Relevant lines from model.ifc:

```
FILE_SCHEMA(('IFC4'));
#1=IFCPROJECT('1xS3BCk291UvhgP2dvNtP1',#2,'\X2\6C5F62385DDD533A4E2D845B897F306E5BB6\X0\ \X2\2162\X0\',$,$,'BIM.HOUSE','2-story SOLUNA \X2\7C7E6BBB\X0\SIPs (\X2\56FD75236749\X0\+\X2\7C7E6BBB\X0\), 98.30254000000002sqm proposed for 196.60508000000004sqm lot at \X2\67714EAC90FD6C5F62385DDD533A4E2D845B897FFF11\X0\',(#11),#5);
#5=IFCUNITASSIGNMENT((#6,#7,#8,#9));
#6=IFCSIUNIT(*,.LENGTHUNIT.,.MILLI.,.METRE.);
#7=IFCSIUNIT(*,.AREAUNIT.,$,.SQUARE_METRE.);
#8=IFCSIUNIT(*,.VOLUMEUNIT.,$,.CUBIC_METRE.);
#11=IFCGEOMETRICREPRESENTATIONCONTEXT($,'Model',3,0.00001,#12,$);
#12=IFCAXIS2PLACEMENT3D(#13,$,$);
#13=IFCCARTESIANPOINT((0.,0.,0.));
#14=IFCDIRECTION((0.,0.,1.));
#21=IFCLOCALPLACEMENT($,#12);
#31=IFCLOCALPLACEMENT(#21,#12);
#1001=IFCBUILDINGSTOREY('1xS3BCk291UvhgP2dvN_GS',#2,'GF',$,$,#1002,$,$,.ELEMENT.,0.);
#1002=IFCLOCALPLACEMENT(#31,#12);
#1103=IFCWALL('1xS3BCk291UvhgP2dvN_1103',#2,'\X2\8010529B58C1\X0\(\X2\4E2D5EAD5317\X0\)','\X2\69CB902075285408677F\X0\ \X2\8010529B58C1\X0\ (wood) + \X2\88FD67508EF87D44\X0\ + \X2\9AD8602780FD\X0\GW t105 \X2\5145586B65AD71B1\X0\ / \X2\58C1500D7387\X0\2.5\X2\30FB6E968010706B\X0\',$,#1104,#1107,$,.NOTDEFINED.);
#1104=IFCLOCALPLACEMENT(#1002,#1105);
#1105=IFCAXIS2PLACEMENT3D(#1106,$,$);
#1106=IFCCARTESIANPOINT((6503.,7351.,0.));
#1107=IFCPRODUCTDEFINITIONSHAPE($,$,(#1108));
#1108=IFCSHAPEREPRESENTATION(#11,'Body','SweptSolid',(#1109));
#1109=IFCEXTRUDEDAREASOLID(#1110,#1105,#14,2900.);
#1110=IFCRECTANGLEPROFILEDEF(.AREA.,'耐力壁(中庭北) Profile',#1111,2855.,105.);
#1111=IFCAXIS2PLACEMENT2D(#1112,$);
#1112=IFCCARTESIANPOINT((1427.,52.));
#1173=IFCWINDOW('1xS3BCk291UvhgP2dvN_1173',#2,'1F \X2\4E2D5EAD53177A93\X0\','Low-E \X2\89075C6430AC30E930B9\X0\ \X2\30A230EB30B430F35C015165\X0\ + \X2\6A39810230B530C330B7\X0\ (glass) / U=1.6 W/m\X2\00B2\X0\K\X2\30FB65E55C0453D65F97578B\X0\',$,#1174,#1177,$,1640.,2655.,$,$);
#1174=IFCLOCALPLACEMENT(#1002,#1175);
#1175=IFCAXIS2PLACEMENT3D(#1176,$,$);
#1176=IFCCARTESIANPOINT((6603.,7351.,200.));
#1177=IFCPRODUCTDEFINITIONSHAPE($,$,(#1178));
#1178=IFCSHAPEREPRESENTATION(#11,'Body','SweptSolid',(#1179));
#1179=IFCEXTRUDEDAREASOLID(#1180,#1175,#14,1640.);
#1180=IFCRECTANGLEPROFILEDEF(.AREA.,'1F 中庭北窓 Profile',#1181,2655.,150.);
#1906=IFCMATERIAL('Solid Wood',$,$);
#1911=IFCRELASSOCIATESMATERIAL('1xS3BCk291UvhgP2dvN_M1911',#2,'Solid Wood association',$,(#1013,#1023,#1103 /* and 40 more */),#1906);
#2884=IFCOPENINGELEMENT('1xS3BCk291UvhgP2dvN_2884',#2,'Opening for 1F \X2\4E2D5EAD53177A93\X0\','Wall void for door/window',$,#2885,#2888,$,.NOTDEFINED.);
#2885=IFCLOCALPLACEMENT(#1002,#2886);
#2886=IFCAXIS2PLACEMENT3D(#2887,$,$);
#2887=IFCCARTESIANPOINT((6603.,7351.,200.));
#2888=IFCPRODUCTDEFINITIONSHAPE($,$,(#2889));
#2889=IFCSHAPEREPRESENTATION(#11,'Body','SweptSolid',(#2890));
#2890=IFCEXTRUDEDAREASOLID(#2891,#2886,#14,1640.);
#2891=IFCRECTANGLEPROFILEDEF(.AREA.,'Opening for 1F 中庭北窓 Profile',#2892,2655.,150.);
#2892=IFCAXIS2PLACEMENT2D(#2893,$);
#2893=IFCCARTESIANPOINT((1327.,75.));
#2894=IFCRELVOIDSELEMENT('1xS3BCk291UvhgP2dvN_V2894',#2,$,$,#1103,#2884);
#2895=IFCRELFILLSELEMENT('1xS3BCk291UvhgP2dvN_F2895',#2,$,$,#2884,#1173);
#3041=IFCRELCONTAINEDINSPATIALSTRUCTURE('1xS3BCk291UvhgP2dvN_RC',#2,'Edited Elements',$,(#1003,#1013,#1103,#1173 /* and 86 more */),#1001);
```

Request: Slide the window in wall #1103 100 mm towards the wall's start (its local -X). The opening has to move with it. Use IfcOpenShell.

```python
import ifcopenshell
import ifcopenshell.api.geometry
import ifcopenshell.util.placement

model = ifcopenshell.open("model.ifc")

window = model.by_guid("1xS3BCk291UvhgP2dvN_1173")
opening = window.FillsVoids[0].RelatingOpeningElement
wall = opening.VoidsElements[0].RelatingBuildingElement

wall_matrix = ifcopenshell.util.placement.get_local_placement(wall.ObjectPlacement)
shift = wall_matrix[:3, 0] * -100.0
before = ifcopenshell.util.placement.get_local_placement(window.ObjectPlacement)[:3, 3].copy()

# The window is not placed relative to its opening, so move both.
for product in (opening, window):
    matrix = ifcopenshell.util.placement.get_local_placement(product.ObjectPlacement)
    matrix[:3, 3] += shift
    ifcopenshell.api.geometry.edit_object_placement(model, product=product, matrix=matrix, is_si=False)

after = ifcopenshell.util.placement.get_local_placement(window.ObjectPlacement)[:3, 3]
print("window moved by", (after - before).round(3) + 0.0)

model.write("model_rev.ifc")
```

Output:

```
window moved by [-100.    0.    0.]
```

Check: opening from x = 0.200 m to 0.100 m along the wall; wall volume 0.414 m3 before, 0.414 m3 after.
